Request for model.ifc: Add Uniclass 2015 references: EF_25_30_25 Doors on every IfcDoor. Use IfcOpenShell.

First a look at what the model holds.

```python
import ifcopenshell

model = ifcopenshell.open("model.ifc")
print(model.schema)
print("classifications:", [c.Name for c in model.by_type("IfcClassification")])
for ifc_class in ("IfcDoor", "IfcRoof", "IfcStair", "IfcWall", "IfcWindow"):
    print(ifc_class, len(model.by_type(ifc_class)))
```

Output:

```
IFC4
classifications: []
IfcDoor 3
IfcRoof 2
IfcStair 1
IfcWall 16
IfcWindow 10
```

```python
import ifcopenshell
import ifcopenshell.api.classification

model = ifcopenshell.open("model.ifc")

system = ifcopenshell.api.classification.add_classification(model, classification="Uniclass 2015")

codes = {
    "IfcDoor": ("EF_25_30_25", "Doors"),
}
for ifc_class, (code, name) in codes.items():
    products = model.by_type(ifc_class)
    ifcopenshell.api.classification.add_reference(
        model, products=products, classification=system, identification=code, name=name
    )
    print(code, len(products))

model.write("model_v2.ifc")
```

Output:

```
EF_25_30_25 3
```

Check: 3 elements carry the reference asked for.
